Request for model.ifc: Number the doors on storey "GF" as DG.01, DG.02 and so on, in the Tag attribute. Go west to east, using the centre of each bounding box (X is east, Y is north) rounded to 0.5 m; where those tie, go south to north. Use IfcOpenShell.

First a look at what the model holds.

```python
import ifcopenshell
import ifcopenshell.util.element
import ifcopenshell.util.placement

model = ifcopenshell.open("model.ifc")
print(model.schema)
storey = next(s for s in model.by_type("IfcBuildingStorey") if s.Name == "GF")
doors = [e for e in ifcopenshell.util.element.get_decomposition(storey) if e.is_a("IfcDoor")]
for e in sorted(doors, key=lambda e: e.id()):
    origin = ifcopenshell.util.placement.get_local_placement(e.ObjectPlacement)[:3, 3]
    print(e.id(), e.Tag, e.Name, origin.round(2) + 0.0, sep=" | ")
```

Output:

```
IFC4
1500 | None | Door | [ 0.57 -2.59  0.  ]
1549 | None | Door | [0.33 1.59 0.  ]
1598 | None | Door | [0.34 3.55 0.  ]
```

```python
import ifcopenshell
import ifcopenshell.geom
import ifcopenshell.util.element
import ifcopenshell.util.shape

model = ifcopenshell.open("model.ifc")
settings = ifcopenshell.geom.settings()
settings.set("use-world-coords", True)


def centre(element):
    shape = ifcopenshell.geom.create_shape(settings, element)
    return ifcopenshell.util.shape.get_bbox_centroid(shape.geometry)


storey = next(s for s in model.by_type("IfcBuildingStorey") if s.Name == "GF")
doors = [e for e in ifcopenshell.util.element.get_decomposition(storey) if e.is_a("IfcDoor")]

# Insertion points can sit at a corner or the storey origin, so sort by the geometry (in metres).
centres = {e: centre(e) for e in doors}
doors.sort(key=lambda e: (round(centres[e][0] / 0.5), centres[e][1]))

for i, e in enumerate(doors, start=1):
    number = f"DG.{i:02d}"
    e.Tag = number
    print(e.id(), number)

model.write("model_v2.ifc")
```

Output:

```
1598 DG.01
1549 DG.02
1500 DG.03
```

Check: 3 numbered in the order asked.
